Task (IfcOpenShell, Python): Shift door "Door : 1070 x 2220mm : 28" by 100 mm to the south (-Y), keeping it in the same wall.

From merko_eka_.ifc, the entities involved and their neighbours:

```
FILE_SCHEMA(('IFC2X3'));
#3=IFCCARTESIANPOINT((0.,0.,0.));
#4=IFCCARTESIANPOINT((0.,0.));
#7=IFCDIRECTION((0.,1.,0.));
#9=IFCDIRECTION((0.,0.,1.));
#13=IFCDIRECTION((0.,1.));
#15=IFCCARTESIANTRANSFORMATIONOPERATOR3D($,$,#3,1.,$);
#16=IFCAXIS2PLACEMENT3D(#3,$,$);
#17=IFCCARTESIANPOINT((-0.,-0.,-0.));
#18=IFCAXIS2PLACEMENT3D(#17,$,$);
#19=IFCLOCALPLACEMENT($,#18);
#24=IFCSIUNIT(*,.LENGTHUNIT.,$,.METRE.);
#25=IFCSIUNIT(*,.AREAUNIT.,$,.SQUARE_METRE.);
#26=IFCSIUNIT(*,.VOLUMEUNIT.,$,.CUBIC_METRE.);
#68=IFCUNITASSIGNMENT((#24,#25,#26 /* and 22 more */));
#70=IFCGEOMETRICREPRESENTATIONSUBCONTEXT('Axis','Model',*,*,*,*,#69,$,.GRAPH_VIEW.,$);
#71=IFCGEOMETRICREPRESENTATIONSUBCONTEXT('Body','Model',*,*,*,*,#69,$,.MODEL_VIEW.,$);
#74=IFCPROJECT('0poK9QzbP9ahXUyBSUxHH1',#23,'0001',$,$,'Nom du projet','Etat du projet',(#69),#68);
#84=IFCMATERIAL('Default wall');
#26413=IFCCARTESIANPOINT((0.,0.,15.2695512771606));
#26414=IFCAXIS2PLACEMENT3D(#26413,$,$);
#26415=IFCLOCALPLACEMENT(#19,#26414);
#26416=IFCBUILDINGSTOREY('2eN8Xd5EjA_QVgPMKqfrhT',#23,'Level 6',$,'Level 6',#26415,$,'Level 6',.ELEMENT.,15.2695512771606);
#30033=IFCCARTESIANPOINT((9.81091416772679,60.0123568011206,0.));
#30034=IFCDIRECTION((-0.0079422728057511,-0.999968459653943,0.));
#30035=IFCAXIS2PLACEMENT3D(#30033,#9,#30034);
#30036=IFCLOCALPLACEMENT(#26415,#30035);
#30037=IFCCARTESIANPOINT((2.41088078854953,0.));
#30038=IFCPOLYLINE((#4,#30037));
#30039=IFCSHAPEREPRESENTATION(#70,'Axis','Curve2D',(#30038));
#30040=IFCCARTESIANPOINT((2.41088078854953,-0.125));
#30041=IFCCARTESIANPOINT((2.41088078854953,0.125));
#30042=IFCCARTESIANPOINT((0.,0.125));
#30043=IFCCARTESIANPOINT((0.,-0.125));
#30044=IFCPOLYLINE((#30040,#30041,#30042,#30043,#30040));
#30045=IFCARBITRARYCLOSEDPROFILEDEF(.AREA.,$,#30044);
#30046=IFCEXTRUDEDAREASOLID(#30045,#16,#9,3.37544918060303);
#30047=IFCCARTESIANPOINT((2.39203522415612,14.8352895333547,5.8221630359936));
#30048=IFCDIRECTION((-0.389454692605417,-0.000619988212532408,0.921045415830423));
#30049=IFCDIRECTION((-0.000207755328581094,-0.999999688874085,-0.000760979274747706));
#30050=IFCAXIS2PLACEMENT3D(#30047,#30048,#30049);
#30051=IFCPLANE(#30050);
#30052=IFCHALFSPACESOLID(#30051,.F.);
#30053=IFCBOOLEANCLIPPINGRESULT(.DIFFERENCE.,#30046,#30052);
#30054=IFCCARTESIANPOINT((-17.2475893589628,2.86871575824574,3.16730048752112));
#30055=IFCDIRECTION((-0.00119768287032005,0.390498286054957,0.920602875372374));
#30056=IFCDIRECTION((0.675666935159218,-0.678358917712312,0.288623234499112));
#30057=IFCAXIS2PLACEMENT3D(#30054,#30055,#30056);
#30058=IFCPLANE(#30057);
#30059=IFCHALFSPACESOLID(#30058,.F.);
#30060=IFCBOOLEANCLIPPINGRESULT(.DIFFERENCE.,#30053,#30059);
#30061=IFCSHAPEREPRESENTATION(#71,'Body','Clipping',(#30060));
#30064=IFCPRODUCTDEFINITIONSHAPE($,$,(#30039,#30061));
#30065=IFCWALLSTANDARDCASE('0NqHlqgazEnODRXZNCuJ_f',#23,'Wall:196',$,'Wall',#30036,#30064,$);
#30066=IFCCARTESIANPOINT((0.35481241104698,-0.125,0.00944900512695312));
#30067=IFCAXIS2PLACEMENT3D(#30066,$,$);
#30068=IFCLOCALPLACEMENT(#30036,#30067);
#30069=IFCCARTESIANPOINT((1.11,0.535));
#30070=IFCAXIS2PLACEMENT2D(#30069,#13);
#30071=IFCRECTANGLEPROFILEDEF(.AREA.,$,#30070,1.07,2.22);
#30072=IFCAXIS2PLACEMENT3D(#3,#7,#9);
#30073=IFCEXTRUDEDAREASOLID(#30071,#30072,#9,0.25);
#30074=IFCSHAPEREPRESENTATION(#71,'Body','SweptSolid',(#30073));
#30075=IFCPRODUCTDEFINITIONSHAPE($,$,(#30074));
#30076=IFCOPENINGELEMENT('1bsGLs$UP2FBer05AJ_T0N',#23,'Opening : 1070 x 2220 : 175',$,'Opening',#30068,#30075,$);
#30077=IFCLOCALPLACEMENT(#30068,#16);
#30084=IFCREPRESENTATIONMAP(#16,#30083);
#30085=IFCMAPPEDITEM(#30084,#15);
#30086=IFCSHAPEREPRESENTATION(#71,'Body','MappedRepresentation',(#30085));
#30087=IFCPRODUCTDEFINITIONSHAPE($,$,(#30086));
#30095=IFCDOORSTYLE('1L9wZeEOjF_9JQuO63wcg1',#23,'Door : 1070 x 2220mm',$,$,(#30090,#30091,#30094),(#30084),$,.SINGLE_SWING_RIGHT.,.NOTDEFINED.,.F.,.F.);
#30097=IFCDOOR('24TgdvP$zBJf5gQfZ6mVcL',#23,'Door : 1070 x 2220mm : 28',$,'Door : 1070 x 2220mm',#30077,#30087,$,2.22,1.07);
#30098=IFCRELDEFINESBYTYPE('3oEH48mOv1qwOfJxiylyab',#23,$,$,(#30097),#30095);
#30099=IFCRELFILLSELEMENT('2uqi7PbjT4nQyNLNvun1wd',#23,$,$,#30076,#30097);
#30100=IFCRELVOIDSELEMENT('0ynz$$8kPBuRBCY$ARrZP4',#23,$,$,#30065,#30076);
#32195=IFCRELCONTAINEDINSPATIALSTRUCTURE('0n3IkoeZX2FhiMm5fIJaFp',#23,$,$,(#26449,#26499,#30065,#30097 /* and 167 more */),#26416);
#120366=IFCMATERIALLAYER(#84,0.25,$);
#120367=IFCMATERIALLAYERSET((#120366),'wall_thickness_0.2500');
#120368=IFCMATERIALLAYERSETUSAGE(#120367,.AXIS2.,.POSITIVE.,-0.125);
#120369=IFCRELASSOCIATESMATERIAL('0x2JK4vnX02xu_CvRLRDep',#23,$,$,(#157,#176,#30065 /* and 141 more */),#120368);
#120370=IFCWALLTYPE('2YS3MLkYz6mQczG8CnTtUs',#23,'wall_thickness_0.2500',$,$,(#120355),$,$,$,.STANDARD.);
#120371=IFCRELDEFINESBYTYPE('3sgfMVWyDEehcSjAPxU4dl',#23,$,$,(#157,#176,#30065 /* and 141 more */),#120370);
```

```python
import ifcopenshell
import ifcopenshell.api.geometry
import ifcopenshell.util.placement

model = ifcopenshell.open("merko_eka_.ifc")

door = model.by_guid("24TgdvP$zBJf5gQfZ6mVcL")
opening = door.FillsVoids[0].RelatingOpeningElement
wall = opening.VoidsElements[0].RelatingBuildingElement

wall_matrix = ifcopenshell.util.placement.get_local_placement(wall.ObjectPlacement)
shift = wall_matrix[:3, 0] * 0.1
before = ifcopenshell.util.placement.get_local_placement(door.ObjectPlacement)[:3, 3].copy()

# The door is placed relative to its opening, so it follows when the opening moves.
matrix = ifcopenshell.util.placement.get_local_placement(opening.ObjectPlacement)
matrix[:3, 3] += shift
ifcopenshell.api.geometry.edit_object_placement(
    model, product=opening, matrix=matrix, is_si=False, should_transform_children=True
)

after = ifcopenshell.util.placement.get_local_placement(door.ObjectPlacement)[:3, 3]
print("door moved by", (after - before).round(3) + 0.0)

model.write("merko_eka__v2.ifc")
```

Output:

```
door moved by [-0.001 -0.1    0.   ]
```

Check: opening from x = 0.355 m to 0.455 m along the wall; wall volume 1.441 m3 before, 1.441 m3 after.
